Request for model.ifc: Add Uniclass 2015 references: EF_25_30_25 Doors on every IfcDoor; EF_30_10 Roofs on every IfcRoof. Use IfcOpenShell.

First a look at what the model holds.

```python
import ifcopenshell

model = ifcopenshell.open("model.ifc")
print(model.schema)
print("classifications:", [c.Name for c in model.by_type("IfcClassification")])
for ifc_class in ("IfcDoor", "IfcRoof", "IfcStair", "IfcWall", "IfcWindow"):
    print(ifc_class, len(model.by_type(ifc_class)))
```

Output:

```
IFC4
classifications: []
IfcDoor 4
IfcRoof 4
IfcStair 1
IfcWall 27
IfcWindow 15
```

```python
import ifcopenshell
import ifcopenshell.api.classification

model = ifcopenshell.open("model.ifc")

system = ifcopenshell.api.classification.add_classification(model, classification="Uniclass 2015")

codes = {
    "IfcDoor": ("EF_25_30_25", "Doors"),
    "IfcRoof": ("EF_30_10", "Roofs"),
}
for ifc_class, (code, name) in codes.items():
    products = model.by_type(ifc_class)
    ifcopenshell.api.classification.add_reference(
        model, products=products, classification=system, identification=code, name=name
    )
    print(code, len(products))

model.write("model_rev.ifc")
```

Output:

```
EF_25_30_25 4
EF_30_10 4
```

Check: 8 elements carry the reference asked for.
